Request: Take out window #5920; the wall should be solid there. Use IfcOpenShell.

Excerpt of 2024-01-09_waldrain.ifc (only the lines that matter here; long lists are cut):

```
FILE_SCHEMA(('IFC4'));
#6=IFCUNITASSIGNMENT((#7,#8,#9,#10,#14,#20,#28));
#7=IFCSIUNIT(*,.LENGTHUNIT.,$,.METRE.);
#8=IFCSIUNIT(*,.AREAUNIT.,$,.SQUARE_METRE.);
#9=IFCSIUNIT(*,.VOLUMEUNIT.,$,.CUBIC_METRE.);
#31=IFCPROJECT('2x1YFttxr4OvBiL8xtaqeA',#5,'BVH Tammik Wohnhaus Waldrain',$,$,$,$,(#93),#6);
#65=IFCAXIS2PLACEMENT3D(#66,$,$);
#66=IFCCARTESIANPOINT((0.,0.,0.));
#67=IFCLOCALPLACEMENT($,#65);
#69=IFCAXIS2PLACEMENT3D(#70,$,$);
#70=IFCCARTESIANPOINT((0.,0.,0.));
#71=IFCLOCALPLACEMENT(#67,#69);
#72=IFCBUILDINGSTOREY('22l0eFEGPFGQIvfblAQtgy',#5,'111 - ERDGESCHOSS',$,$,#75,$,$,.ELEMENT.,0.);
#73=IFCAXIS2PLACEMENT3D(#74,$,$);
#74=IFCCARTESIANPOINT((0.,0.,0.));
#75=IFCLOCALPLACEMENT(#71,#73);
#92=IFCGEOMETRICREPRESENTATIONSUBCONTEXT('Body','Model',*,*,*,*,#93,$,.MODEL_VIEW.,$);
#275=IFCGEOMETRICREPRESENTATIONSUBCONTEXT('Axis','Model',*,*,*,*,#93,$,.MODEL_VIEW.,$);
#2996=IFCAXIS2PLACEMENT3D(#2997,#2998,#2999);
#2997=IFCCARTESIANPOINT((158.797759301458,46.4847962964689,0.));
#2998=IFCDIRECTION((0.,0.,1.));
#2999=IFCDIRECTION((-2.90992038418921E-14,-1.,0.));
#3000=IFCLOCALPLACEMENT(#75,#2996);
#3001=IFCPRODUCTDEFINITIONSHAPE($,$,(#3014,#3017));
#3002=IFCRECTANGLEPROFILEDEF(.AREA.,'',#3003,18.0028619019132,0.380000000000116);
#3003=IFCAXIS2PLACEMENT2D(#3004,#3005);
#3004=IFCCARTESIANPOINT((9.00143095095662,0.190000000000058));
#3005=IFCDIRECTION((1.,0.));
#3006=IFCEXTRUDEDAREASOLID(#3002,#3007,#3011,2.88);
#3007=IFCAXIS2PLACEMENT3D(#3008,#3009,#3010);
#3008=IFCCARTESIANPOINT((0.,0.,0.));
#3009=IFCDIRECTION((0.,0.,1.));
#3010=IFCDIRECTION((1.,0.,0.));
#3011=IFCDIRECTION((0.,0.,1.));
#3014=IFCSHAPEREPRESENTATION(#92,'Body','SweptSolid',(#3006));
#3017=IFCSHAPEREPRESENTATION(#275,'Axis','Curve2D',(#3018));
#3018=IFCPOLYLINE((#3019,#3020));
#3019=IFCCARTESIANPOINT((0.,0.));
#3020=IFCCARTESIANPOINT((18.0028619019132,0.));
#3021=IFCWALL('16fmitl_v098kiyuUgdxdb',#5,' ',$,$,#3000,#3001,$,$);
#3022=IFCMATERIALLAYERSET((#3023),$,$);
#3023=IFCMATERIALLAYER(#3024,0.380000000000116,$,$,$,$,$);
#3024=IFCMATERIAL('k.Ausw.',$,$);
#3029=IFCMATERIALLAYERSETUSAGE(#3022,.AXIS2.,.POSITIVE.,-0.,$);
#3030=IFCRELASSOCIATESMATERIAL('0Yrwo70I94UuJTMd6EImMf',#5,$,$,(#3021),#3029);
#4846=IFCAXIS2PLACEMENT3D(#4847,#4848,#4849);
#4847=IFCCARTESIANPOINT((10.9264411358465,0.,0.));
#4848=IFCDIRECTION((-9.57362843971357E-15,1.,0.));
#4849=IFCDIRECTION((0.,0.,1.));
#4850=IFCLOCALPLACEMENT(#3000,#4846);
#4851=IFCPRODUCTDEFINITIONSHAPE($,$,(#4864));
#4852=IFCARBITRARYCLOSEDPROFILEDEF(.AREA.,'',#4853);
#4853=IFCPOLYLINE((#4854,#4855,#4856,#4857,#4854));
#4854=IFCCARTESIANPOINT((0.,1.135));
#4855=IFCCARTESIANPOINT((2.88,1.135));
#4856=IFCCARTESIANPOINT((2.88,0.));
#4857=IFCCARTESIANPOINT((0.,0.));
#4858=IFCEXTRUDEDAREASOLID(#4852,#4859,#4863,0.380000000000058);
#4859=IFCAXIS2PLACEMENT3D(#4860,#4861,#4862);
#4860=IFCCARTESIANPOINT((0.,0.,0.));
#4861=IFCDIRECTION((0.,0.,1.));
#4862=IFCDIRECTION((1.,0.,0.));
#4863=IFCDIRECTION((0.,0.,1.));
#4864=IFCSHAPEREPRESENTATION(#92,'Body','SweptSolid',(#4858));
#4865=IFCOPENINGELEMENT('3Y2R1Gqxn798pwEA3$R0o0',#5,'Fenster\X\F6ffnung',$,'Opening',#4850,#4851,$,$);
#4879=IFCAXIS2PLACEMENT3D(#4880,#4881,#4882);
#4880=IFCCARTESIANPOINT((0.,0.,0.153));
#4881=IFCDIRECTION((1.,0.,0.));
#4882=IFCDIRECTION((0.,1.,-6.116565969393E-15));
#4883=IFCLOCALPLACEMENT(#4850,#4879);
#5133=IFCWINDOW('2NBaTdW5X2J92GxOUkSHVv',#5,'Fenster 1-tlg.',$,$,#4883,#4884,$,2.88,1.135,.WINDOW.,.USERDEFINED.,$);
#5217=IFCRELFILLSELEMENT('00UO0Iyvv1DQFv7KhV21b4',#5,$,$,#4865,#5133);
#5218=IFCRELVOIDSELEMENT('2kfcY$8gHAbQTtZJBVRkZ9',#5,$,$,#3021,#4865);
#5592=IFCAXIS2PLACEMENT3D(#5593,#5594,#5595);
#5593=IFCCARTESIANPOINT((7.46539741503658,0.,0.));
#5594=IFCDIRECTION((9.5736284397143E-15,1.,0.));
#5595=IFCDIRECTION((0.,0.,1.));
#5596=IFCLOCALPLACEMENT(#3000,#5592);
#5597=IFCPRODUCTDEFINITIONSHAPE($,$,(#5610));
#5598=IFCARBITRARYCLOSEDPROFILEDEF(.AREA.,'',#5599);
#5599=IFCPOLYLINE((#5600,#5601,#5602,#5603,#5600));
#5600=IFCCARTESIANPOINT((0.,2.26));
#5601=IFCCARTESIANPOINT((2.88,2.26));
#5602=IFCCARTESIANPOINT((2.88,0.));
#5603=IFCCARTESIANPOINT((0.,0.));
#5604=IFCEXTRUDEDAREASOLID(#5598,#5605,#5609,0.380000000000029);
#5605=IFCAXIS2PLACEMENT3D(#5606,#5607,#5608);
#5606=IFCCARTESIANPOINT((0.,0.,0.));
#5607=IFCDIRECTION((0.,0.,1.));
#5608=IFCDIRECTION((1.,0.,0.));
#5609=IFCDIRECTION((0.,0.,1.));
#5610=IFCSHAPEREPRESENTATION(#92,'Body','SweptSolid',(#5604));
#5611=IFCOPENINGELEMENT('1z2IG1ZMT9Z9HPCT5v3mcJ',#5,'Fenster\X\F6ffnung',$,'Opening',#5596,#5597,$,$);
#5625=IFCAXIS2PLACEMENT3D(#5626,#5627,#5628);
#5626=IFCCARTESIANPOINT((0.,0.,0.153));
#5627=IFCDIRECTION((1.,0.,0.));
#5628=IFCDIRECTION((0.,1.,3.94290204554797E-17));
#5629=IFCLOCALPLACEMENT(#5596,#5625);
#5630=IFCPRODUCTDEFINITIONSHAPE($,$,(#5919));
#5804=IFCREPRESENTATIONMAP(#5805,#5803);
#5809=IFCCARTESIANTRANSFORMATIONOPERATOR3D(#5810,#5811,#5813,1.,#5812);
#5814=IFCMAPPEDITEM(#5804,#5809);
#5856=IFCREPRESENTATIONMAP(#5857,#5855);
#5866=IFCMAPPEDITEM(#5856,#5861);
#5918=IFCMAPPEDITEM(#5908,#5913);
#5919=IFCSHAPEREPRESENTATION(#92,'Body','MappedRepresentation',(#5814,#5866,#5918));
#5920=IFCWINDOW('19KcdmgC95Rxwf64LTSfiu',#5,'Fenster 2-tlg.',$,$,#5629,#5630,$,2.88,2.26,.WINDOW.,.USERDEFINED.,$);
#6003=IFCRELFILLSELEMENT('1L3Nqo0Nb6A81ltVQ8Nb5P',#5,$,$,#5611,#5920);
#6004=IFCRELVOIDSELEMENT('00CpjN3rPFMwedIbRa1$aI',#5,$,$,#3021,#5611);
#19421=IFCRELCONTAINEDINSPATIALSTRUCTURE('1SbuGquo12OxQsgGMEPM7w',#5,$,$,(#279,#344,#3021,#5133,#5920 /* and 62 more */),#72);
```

```python
import ifcopenshell
import ifcopenshell.api.feature
import ifcopenshell.api.root
import ifcopenshell.geom
import ifcopenshell.util.shape

model = ifcopenshell.open("2024-01-09_waldrain.ifc")
settings = ifcopenshell.geom.settings()


def volume(element):
    """Net volume in cubic metres, openings subtracted."""
    shape = ifcopenshell.geom.create_shape(settings, element)
    return ifcopenshell.util.shape.get_volume(shape.geometry)


window = model.by_id(5920)
opening = window.FillsVoids[0].RelatingOpeningElement
wall = opening.VoidsElements[0].RelatingBuildingElement
before = volume(wall)

ifcopenshell.api.root.remove_product(model, product=window)
ifcopenshell.api.feature.remove_feature(model, feature=opening)

after = volume(wall)

print(f"wall volume {before:.3f} -> {after:.3f} m3")

model.write("2024-01-09_waldrain_edited.ifc")
```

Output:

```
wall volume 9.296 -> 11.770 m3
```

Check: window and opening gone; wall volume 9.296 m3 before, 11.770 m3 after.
